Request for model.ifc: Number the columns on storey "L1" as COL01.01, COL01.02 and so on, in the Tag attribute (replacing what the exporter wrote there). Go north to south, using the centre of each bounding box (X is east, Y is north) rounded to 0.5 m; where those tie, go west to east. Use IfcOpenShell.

First a look at what the model holds.

```python
import ifcopenshell
import ifcopenshell.util.element
import ifcopenshell.util.placement

model = ifcopenshell.open("model.ifc")
print(model.schema)
storey = next(s for s in model.by_type("IfcBuildingStorey") if s.Name == "L1")
columns = [e for e in ifcopenshell.util.element.get_decomposition(storey) if e.is_a("IfcColumn")]
for e in sorted(columns, key=lambda e: e.id()):
    origin = ifcopenshell.util.placement.get_local_placement(e.ObjectPlacement)[:3, 3]
    print(e.id(), e.Tag, e.Name, origin.round(2) + 0.0, sep=" | ")
```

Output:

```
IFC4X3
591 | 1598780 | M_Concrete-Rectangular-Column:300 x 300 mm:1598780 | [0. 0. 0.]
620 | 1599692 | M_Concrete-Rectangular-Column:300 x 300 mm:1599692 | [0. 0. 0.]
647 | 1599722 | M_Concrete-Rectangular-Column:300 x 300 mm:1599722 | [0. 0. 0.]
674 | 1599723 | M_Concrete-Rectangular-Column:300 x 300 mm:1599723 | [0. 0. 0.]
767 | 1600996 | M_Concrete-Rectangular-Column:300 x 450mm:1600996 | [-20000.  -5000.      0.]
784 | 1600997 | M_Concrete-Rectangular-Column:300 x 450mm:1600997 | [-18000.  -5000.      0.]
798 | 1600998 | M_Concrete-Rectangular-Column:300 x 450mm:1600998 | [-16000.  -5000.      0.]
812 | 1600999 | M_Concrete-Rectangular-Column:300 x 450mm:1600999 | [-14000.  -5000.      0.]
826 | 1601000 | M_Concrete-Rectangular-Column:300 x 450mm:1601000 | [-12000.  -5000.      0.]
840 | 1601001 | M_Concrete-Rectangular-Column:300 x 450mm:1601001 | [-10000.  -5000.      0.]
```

```python
import ifcopenshell
import ifcopenshell.geom
import ifcopenshell.util.element
import ifcopenshell.util.shape

model = ifcopenshell.open("model.ifc")
settings = ifcopenshell.geom.settings()
settings.set("use-world-coords", True)


def centre(element):
    shape = ifcopenshell.geom.create_shape(settings, element)
    return ifcopenshell.util.shape.get_bbox_centroid(shape.geometry)


storey = next(s for s in model.by_type("IfcBuildingStorey") if s.Name == "L1")
columns = [e for e in ifcopenshell.util.element.get_decomposition(storey) if e.is_a("IfcColumn")]

# Insertion points can sit at a corner or the storey origin, so sort by the geometry (in metres).
centres = {e: centre(e) for e in columns}
columns.sort(key=lambda e: (-round(centres[e][1] / 0.5), centres[e][0]))

for i, e in enumerate(columns, start=1):
    number = f"COL01.{i:02d}"
    e.Tag = number
    print(e.id(), number)

model.write("model_rev.ifc")
```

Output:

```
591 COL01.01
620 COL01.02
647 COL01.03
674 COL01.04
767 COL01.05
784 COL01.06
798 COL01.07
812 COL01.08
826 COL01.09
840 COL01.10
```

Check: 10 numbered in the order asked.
